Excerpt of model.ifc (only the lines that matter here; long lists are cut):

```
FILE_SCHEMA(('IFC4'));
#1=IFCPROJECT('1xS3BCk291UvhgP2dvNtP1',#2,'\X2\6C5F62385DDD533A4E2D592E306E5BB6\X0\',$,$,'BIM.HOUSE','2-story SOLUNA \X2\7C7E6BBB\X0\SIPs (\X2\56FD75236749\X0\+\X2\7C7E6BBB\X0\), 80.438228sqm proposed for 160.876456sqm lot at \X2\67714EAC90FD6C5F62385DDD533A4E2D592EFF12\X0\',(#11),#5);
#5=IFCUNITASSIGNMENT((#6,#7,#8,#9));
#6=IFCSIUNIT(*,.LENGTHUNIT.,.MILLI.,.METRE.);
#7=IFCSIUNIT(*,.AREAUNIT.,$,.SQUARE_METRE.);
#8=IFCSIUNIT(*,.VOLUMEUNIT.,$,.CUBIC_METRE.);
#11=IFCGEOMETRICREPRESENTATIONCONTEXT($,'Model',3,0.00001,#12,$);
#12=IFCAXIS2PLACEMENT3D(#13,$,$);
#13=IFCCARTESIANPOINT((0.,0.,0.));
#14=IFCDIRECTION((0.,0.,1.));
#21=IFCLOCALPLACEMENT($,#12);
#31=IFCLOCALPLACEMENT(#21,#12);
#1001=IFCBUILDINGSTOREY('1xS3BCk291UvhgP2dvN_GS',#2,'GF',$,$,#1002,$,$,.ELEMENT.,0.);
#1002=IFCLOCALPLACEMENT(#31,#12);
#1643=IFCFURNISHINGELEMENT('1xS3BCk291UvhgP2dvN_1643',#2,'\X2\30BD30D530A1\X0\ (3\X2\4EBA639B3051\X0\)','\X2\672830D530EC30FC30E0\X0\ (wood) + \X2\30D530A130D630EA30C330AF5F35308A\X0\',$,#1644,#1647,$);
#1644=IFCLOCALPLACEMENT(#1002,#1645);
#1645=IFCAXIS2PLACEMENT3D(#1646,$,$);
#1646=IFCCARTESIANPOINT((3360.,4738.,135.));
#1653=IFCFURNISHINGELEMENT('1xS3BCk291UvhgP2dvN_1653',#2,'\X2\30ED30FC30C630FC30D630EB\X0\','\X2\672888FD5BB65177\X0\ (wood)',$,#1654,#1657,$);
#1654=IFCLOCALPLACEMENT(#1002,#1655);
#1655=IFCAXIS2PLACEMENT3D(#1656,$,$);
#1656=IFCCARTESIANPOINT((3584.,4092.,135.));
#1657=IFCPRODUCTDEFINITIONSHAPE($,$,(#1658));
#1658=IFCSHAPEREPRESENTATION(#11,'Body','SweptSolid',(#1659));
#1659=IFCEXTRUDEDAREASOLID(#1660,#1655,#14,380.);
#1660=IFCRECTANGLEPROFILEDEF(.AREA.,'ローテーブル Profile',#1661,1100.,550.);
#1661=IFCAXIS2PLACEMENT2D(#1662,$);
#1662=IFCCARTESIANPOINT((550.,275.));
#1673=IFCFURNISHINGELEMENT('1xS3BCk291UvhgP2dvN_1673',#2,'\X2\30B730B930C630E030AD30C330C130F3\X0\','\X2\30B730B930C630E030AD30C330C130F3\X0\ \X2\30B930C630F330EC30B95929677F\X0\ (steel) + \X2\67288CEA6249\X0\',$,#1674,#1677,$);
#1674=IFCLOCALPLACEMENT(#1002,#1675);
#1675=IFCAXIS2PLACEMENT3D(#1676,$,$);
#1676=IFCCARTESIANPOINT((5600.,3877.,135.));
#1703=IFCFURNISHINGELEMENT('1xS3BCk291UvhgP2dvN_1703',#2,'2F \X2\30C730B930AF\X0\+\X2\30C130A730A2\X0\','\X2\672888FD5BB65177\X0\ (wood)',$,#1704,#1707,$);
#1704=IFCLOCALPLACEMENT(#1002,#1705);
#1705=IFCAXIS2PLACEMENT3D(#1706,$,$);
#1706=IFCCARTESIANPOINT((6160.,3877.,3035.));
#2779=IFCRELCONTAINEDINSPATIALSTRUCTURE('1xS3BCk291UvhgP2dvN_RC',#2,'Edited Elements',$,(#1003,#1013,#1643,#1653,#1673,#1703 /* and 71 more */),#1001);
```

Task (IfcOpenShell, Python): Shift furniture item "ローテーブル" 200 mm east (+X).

```python
import ifcopenshell
import ifcopenshell.api.geometry
import ifcopenshell.util.placement
import ifcopenshell.util.unit

model = ifcopenshell.open("model.ifc")
unit_scale = ifcopenshell.util.unit.calculate_unit_scale(model)

item = model.by_guid("1xS3BCk291UvhgP2dvN_1653")
matrix = ifcopenshell.util.placement.get_local_placement(item.ObjectPlacement)
matrix[0, 3] += 0.2 / unit_scale
ifcopenshell.api.geometry.edit_object_placement(model, product=item, matrix=matrix, is_si=False)

print(ifcopenshell.util.placement.get_local_placement(item.ObjectPlacement).round(3) + 0.0)

model.write("model_edited.ifc")
```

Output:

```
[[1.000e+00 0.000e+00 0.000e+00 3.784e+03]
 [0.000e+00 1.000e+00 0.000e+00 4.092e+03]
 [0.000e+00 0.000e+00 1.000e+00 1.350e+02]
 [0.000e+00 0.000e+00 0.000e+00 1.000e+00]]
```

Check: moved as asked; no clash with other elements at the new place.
